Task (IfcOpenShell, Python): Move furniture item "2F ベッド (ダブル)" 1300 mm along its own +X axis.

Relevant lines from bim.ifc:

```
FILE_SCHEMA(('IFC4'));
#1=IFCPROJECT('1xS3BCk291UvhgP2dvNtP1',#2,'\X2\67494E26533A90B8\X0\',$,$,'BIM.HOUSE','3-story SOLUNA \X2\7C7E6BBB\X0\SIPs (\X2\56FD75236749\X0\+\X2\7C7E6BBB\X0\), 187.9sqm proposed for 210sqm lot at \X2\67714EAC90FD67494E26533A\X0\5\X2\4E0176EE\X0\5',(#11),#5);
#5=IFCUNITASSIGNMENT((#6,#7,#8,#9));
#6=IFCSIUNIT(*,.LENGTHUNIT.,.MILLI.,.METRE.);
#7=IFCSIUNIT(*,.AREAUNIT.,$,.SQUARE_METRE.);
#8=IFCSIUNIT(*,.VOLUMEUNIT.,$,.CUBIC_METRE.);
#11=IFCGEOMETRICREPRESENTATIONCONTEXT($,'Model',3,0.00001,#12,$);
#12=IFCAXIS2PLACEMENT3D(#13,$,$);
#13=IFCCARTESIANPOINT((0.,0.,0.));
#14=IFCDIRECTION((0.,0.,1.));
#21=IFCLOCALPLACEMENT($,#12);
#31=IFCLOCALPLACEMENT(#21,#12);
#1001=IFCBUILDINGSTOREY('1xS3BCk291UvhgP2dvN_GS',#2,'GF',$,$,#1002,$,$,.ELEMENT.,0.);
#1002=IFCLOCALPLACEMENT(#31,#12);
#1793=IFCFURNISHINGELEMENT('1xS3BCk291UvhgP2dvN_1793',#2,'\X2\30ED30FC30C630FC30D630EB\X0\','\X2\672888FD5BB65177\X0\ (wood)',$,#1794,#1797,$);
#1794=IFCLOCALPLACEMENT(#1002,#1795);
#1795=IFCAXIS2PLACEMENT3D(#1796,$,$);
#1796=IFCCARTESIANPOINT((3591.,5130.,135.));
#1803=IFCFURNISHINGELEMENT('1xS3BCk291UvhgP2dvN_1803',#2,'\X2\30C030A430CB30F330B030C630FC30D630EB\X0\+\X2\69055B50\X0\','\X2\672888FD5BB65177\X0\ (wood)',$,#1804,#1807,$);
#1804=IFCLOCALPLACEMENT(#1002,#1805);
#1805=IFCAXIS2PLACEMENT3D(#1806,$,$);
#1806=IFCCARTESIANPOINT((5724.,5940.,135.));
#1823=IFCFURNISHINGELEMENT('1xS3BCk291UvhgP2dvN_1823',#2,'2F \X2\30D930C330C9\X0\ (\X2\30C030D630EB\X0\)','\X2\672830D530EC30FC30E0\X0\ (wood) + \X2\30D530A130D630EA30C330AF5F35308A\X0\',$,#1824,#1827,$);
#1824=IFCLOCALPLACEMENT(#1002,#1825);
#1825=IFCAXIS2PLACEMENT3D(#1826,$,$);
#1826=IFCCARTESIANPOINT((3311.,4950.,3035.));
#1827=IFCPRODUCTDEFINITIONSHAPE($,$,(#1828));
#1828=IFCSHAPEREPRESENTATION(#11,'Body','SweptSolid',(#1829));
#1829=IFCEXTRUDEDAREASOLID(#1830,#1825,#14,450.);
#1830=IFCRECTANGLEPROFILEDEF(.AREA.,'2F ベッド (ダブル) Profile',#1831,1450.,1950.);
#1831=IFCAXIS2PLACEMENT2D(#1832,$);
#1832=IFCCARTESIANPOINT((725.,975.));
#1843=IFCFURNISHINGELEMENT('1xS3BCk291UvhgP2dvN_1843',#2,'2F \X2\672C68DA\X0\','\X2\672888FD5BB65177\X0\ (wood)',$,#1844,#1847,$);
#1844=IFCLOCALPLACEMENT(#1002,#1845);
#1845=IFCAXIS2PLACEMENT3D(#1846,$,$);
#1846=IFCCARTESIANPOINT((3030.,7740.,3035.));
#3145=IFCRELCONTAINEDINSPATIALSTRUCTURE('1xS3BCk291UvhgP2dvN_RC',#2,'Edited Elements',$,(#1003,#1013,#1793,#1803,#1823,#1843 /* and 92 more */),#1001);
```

```python
import ifcopenshell
import ifcopenshell.api.geometry
import ifcopenshell.util.placement
import ifcopenshell.util.unit

model = ifcopenshell.open("bim.ifc")
unit_scale = ifcopenshell.util.unit.calculate_unit_scale(model)

item = model.by_guid("1xS3BCk291UvhgP2dvN_1823")
matrix = ifcopenshell.util.placement.get_local_placement(item.ObjectPlacement)
matrix[:3, 3] += matrix[:3, 0] * 1.3 / unit_scale
ifcopenshell.api.geometry.edit_object_placement(model, product=item, matrix=matrix, is_si=False)

print(ifcopenshell.util.placement.get_local_placement(item.ObjectPlacement).round(3) + 0.0)

model.write("bim_updated.ifc")
```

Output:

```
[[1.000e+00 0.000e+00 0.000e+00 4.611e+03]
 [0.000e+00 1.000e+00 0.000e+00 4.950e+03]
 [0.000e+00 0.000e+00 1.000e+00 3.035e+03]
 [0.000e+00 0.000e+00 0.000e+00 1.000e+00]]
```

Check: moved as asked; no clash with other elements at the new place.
